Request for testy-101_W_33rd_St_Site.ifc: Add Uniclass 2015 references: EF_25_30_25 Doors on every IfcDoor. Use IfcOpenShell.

First a look at what the model holds.

```python
import ifcopenshell

model = ifcopenshell.open("testy-101_W_33rd_St_Site.ifc")
print(model.schema)
print("classifications:", [c.Name for c in model.by_type("IfcClassification")])
for ifc_class in ("IfcDoor", "IfcRoof", "IfcStair", "IfcWall", "IfcWindow"):
    print(ifc_class, len(model.by_type(ifc_class)))
```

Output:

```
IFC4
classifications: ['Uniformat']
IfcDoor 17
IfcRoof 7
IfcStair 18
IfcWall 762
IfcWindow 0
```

```python
import ifcopenshell
import ifcopenshell.api.classification

model = ifcopenshell.open("testy-101_W_33rd_St_Site.ifc")

system = ifcopenshell.api.classification.add_classification(model, classification="Uniclass 2015")

codes = {
    "IfcDoor": ("EF_25_30_25", "Doors"),
}
for ifc_class, (code, name) in codes.items():
    products = model.by_type(ifc_class)
    ifcopenshell.api.classification.add_reference(
        model, products=products, classification=system, identification=code, name=name
    )
    print(code, len(products))

model.write("testy-101_W_33rd_St_Site_rev.ifc")
```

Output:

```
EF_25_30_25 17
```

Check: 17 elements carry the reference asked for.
